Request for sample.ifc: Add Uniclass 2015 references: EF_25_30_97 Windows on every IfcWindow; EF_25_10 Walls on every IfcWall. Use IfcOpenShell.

First a look at what the model holds.

```python
import ifcopenshell

model = ifcopenshell.open("sample.ifc")
print(model.schema)
print("classifications:", [c.Name for c in model.by_type("IfcClassification")])
for ifc_class in ("IfcDoor", "IfcRoof", "IfcStair", "IfcWall", "IfcWindow"):
    print(ifc_class, len(model.by_type(ifc_class)))
```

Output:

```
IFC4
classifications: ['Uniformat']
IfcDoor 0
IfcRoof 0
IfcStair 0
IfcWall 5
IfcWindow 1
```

```python
import ifcopenshell
import ifcopenshell.api.classification

model = ifcopenshell.open("sample.ifc")

system = ifcopenshell.api.classification.add_classification(model, classification="Uniclass 2015")

codes = {
    "IfcWindow": ("EF_25_30_97", "Windows"),
    "IfcWall": ("EF_25_10", "Walls"),
}
for ifc_class, (code, name) in codes.items():
    products = model.by_type(ifc_class)
    ifcopenshell.api.classification.add_reference(
        model, products=products, classification=system, identification=code, name=name
    )
    print(code, len(products))

model.write("sample_rev.ifc")
```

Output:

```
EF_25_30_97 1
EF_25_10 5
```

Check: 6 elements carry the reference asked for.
